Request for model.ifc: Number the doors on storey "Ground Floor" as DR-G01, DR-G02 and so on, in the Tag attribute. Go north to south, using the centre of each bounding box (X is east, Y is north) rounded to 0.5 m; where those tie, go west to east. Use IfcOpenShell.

First a look at what the model holds.

```python
import ifcopenshell
import ifcopenshell.util.element
import ifcopenshell.util.placement

model = ifcopenshell.open("model.ifc")
print(model.schema)
storey = next(s for s in model.by_type("IfcBuildingStorey") if s.Name == "Ground Floor")
doors = [e for e in ifcopenshell.util.element.get_decomposition(storey) if e.is_a("IfcDoor")]
for e in sorted(doors, key=lambda e: e.id()):
    origin = ifcopenshell.util.placement.get_local_placement(e.ObjectPlacement)[:3, 3]
    print(e.id(), e.Tag, e.Name, origin.round(2) + 0.0, sep=" | ")
```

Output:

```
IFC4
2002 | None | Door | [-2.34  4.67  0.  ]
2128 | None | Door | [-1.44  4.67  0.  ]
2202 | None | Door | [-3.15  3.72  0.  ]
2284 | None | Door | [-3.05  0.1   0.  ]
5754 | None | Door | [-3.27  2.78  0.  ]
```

```python
import ifcopenshell
import ifcopenshell.geom
import ifcopenshell.util.element
import ifcopenshell.util.shape

model = ifcopenshell.open("model.ifc")
settings = ifcopenshell.geom.settings()
settings.set("use-world-coords", True)


def centre(element):
    shape = ifcopenshell.geom.create_shape(settings, element)
    return ifcopenshell.util.shape.get_bbox_centroid(shape.geometry)


storey = next(s for s in model.by_type("IfcBuildingStorey") if s.Name == "Ground Floor")
doors = [e for e in ifcopenshell.util.element.get_decomposition(storey) if e.is_a("IfcDoor")]

# Insertion points can sit at a corner or the storey origin, so sort by the geometry (in metres).
centres = {e: centre(e) for e in doors}
doors.sort(key=lambda e: (-round(centres[e][1] / 0.5), centres[e][0]))

for i, e in enumerate(doors, start=1):
    number = f"DR-G{i:02d}"
    e.Tag = number
    print(e.id(), number)

model.write("model_edited.ifc")
```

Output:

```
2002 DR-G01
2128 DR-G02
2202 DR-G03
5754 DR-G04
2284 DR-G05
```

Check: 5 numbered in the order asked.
